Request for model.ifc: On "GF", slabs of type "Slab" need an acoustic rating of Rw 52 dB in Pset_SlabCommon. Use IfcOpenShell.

First a look at what the model holds.

```python
import ifcopenshell
import ifcopenshell.util.element

model = ifcopenshell.open("model.ifc")
print(model.schema)
storey = next(s for s in model.by_type("IfcBuildingStorey") if s.Name == "GF")
slabs = [e for e in ifcopenshell.util.element.get_decomposition(storey) if e.is_a("IfcSlab")]
seen = {}
for e in slabs:
    element_type = ifcopenshell.util.element.get_type(e)
    key = (element_type.Name if element_type != e and element_type else None, ifcopenshell.util.element.get_pset(e, "Pset_SlabCommon", "AcousticRating"))
    seen[key] = seen.get(key, 0) + 1
for (name, value), count in sorted(seen.items(), key=str):
    print(count, "x", name, "|", value)
```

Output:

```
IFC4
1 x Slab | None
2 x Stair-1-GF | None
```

```python
import ifcopenshell
import ifcopenshell.api.pset
import ifcopenshell.util.element

model = ifcopenshell.open("model.ifc")

storey = next(s for s in model.by_type("IfcBuildingStorey") if s.Name == "GF")
slabs = [e for e in ifcopenshell.util.element.get_decomposition(storey) if e.is_a("IfcSlab")]

count = 0
for e in slabs:
    element_type = ifcopenshell.util.element.get_type(e)
    if element_type in (None, e) or element_type.Name != "Slab":
        continue
    # add_pset returns the element's existing set when there is one.
    pset = ifcopenshell.api.pset.add_pset(model, product=e, name="Pset_SlabCommon")
    ifcopenshell.api.pset.edit_pset(model, pset=pset, properties={"AcousticRating": "Rw 52 dB"})
    count += 1

print(count, "slabs updated")

model.write("model_edited.ifc")
```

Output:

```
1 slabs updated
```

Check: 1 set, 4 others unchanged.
